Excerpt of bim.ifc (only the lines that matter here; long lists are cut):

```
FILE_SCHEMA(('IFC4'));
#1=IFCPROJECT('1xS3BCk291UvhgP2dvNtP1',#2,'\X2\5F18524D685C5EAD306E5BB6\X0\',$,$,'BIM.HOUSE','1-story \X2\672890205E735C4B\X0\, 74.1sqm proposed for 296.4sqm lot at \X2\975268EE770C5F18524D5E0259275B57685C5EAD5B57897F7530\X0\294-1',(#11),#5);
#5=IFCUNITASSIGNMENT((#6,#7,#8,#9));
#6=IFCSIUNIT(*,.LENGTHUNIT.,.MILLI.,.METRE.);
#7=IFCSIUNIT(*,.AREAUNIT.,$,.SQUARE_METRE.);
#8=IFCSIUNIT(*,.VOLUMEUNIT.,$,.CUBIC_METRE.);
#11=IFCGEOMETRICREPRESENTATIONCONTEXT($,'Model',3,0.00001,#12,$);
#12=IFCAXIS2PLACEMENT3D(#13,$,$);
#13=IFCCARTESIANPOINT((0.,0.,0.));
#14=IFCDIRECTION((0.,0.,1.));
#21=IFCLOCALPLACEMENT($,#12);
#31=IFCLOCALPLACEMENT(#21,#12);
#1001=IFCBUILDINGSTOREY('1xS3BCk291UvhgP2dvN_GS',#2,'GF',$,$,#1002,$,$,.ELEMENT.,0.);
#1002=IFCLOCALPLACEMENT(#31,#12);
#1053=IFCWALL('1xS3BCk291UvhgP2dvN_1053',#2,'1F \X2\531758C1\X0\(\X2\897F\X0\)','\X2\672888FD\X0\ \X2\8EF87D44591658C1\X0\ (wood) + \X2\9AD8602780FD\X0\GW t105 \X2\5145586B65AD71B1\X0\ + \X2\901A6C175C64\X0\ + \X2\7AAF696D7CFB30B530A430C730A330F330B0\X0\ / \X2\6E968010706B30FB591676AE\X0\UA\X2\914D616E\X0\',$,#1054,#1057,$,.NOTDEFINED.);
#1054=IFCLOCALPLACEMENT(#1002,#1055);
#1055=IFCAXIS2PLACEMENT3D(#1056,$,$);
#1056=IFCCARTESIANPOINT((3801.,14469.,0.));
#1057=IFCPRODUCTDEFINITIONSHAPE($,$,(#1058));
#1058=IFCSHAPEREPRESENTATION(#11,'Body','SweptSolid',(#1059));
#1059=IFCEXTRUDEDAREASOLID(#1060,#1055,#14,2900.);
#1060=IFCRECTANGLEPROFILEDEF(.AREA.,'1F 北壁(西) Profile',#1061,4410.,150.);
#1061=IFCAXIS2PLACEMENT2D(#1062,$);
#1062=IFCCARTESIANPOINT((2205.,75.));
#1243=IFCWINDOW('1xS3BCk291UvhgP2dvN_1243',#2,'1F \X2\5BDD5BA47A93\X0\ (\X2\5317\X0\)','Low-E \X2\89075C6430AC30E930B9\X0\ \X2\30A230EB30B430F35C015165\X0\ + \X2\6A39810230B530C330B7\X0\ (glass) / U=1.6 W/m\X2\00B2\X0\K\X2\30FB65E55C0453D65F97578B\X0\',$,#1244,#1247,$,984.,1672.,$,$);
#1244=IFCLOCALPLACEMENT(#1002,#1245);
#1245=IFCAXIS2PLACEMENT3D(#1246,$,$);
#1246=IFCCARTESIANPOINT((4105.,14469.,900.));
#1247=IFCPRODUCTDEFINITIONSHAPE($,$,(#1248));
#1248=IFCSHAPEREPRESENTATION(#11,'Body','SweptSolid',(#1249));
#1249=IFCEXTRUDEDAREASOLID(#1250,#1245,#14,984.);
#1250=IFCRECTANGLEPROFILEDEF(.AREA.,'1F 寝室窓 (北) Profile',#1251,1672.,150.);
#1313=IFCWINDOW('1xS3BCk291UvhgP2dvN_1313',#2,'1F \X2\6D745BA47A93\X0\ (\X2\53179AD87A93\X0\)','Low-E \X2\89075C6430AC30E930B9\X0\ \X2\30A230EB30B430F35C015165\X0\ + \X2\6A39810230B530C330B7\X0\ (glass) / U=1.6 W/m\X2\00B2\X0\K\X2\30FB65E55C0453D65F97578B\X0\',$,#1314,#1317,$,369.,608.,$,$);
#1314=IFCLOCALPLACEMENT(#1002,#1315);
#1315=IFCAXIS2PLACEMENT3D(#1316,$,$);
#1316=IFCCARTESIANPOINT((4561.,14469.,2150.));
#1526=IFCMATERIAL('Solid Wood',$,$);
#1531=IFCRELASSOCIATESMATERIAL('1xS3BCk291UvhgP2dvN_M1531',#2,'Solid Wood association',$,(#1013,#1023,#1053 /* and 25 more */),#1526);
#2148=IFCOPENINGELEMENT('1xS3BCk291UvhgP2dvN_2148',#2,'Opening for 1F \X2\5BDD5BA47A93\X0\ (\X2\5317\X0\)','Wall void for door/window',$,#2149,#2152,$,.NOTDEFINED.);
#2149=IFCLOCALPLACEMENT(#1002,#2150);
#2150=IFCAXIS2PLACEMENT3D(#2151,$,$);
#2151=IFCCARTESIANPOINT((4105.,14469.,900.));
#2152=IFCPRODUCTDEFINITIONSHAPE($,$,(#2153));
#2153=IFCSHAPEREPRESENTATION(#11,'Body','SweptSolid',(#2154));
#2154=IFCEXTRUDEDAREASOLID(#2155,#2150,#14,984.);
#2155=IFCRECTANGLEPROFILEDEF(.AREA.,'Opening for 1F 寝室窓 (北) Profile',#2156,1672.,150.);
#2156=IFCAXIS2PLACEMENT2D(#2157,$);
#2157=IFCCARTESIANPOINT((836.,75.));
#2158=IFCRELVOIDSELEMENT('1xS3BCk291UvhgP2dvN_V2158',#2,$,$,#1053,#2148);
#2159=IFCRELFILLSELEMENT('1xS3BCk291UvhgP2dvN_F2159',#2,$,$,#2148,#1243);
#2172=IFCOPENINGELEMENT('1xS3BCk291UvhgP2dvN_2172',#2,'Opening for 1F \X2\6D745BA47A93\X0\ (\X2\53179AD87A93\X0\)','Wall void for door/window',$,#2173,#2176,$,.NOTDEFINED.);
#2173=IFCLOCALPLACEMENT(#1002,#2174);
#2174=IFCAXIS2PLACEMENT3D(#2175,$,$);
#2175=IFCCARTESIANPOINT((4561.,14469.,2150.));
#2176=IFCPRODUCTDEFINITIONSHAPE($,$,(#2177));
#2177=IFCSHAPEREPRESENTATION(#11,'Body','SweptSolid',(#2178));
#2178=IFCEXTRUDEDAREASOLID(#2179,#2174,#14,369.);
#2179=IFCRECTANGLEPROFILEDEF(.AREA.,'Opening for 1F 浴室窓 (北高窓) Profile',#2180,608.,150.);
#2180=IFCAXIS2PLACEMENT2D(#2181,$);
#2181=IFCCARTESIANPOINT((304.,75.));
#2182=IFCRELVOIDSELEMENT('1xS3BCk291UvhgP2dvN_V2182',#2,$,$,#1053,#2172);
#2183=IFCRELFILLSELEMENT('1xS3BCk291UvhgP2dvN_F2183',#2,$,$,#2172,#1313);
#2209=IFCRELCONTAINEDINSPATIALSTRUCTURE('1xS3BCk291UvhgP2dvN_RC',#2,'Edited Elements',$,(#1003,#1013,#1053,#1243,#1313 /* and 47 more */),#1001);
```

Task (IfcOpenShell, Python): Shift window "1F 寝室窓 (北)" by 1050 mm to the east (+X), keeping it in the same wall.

```python
import ifcopenshell
import ifcopenshell.api.geometry
import ifcopenshell.util.placement

model = ifcopenshell.open("bim.ifc")

window = model.by_guid("1xS3BCk291UvhgP2dvN_1243")
opening = window.FillsVoids[0].RelatingOpeningElement
wall = opening.VoidsElements[0].RelatingBuildingElement

wall_matrix = ifcopenshell.util.placement.get_local_placement(wall.ObjectPlacement)
shift = wall_matrix[:3, 0] * 1050.0
before = ifcopenshell.util.placement.get_local_placement(window.ObjectPlacement)[:3, 3].copy()

# The window is not placed relative to its opening, so move both.
for product in (opening, window):
    matrix = ifcopenshell.util.placement.get_local_placement(product.ObjectPlacement)
    matrix[:3, 3] += shift
    ifcopenshell.api.geometry.edit_object_placement(model, product=product, matrix=matrix, is_si=False)

after = ifcopenshell.util.placement.get_local_placement(window.ObjectPlacement)[:3, 3]
print("window moved by", (after - before).round(3) + 0.0)

model.write("bim_edited.ifc")
```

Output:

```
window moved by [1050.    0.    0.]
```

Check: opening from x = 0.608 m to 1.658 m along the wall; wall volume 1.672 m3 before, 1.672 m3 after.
